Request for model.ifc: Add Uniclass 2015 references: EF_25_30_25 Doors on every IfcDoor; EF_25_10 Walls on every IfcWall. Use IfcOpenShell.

First a look at what the model holds.

```python
import ifcopenshell

model = ifcopenshell.open("model.ifc")
print(model.schema)
print("classifications:", [c.Name for c in model.by_type("IfcClassification")])
for ifc_class in ("IfcDoor", "IfcRoof", "IfcStair", "IfcWall", "IfcWindow"):
    print(ifc_class, len(model.by_type(ifc_class)))
```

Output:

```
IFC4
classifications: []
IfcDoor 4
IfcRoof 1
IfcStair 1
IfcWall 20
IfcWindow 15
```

```python
import ifcopenshell
import ifcopenshell.api.classification

model = ifcopenshell.open("model.ifc")

system = ifcopenshell.api.classification.add_classification(model, classification="Uniclass 2015")

codes = {
    "IfcDoor": ("EF_25_30_25", "Doors"),
    "IfcWall": ("EF_25_10", "Walls"),
}
for ifc_class, (code, name) in codes.items():
    products = model.by_type(ifc_class)
    ifcopenshell.api.classification.add_reference(
        model, products=products, classification=system, identification=code, name=name
    )
    print(code, len(products))

model.write("model_edited.ifc")
```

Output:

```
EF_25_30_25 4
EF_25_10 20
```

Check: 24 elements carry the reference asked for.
